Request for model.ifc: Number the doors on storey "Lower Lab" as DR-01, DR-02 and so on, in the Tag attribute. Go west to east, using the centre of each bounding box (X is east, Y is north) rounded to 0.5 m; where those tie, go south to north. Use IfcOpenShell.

First a look at what the model holds.

```python
import ifcopenshell
import ifcopenshell.util.element
import ifcopenshell.util.placement

model = ifcopenshell.open("model.ifc")
print(model.schema)
storey = next(s for s in model.by_type("IfcBuildingStorey") if s.Name == "Lower Lab")
doors = [e for e in ifcopenshell.util.element.get_decomposition(storey) if e.is_a("IfcDoor")]
for e in sorted(doors, key=lambda e: e.id()):
    origin = ifcopenshell.util.placement.get_local_placement(e.ObjectPlacement)[:3, 3]
    print(e.id(), e.Tag, e.Name, origin.round(2) + 0.0, sep=" | ")
```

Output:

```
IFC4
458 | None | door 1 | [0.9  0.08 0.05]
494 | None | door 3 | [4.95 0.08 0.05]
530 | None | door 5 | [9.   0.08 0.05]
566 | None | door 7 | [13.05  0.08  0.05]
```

```python
import ifcopenshell
import ifcopenshell.geom
import ifcopenshell.util.element
import ifcopenshell.util.shape

model = ifcopenshell.open("model.ifc")
settings = ifcopenshell.geom.settings()
settings.set("use-world-coords", True)


def centre(element):
    shape = ifcopenshell.geom.create_shape(settings, element)
    return ifcopenshell.util.shape.get_bbox_centroid(shape.geometry)


storey = next(s for s in model.by_type("IfcBuildingStorey") if s.Name == "Lower Lab")
doors = [e for e in ifcopenshell.util.element.get_decomposition(storey) if e.is_a("IfcDoor")]

# Insertion points can sit at a corner or the storey origin, so sort by the geometry (in metres).
centres = {e: centre(e) for e in doors}
doors.sort(key=lambda e: (round(centres[e][0] / 0.5), centres[e][1]))

for i, e in enumerate(doors, start=1):
    number = f"DR-{i:02d}"
    e.Tag = number
    print(e.id(), number)

model.write("model_updated.ifc")
```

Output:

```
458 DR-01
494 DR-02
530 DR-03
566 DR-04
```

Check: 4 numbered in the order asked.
